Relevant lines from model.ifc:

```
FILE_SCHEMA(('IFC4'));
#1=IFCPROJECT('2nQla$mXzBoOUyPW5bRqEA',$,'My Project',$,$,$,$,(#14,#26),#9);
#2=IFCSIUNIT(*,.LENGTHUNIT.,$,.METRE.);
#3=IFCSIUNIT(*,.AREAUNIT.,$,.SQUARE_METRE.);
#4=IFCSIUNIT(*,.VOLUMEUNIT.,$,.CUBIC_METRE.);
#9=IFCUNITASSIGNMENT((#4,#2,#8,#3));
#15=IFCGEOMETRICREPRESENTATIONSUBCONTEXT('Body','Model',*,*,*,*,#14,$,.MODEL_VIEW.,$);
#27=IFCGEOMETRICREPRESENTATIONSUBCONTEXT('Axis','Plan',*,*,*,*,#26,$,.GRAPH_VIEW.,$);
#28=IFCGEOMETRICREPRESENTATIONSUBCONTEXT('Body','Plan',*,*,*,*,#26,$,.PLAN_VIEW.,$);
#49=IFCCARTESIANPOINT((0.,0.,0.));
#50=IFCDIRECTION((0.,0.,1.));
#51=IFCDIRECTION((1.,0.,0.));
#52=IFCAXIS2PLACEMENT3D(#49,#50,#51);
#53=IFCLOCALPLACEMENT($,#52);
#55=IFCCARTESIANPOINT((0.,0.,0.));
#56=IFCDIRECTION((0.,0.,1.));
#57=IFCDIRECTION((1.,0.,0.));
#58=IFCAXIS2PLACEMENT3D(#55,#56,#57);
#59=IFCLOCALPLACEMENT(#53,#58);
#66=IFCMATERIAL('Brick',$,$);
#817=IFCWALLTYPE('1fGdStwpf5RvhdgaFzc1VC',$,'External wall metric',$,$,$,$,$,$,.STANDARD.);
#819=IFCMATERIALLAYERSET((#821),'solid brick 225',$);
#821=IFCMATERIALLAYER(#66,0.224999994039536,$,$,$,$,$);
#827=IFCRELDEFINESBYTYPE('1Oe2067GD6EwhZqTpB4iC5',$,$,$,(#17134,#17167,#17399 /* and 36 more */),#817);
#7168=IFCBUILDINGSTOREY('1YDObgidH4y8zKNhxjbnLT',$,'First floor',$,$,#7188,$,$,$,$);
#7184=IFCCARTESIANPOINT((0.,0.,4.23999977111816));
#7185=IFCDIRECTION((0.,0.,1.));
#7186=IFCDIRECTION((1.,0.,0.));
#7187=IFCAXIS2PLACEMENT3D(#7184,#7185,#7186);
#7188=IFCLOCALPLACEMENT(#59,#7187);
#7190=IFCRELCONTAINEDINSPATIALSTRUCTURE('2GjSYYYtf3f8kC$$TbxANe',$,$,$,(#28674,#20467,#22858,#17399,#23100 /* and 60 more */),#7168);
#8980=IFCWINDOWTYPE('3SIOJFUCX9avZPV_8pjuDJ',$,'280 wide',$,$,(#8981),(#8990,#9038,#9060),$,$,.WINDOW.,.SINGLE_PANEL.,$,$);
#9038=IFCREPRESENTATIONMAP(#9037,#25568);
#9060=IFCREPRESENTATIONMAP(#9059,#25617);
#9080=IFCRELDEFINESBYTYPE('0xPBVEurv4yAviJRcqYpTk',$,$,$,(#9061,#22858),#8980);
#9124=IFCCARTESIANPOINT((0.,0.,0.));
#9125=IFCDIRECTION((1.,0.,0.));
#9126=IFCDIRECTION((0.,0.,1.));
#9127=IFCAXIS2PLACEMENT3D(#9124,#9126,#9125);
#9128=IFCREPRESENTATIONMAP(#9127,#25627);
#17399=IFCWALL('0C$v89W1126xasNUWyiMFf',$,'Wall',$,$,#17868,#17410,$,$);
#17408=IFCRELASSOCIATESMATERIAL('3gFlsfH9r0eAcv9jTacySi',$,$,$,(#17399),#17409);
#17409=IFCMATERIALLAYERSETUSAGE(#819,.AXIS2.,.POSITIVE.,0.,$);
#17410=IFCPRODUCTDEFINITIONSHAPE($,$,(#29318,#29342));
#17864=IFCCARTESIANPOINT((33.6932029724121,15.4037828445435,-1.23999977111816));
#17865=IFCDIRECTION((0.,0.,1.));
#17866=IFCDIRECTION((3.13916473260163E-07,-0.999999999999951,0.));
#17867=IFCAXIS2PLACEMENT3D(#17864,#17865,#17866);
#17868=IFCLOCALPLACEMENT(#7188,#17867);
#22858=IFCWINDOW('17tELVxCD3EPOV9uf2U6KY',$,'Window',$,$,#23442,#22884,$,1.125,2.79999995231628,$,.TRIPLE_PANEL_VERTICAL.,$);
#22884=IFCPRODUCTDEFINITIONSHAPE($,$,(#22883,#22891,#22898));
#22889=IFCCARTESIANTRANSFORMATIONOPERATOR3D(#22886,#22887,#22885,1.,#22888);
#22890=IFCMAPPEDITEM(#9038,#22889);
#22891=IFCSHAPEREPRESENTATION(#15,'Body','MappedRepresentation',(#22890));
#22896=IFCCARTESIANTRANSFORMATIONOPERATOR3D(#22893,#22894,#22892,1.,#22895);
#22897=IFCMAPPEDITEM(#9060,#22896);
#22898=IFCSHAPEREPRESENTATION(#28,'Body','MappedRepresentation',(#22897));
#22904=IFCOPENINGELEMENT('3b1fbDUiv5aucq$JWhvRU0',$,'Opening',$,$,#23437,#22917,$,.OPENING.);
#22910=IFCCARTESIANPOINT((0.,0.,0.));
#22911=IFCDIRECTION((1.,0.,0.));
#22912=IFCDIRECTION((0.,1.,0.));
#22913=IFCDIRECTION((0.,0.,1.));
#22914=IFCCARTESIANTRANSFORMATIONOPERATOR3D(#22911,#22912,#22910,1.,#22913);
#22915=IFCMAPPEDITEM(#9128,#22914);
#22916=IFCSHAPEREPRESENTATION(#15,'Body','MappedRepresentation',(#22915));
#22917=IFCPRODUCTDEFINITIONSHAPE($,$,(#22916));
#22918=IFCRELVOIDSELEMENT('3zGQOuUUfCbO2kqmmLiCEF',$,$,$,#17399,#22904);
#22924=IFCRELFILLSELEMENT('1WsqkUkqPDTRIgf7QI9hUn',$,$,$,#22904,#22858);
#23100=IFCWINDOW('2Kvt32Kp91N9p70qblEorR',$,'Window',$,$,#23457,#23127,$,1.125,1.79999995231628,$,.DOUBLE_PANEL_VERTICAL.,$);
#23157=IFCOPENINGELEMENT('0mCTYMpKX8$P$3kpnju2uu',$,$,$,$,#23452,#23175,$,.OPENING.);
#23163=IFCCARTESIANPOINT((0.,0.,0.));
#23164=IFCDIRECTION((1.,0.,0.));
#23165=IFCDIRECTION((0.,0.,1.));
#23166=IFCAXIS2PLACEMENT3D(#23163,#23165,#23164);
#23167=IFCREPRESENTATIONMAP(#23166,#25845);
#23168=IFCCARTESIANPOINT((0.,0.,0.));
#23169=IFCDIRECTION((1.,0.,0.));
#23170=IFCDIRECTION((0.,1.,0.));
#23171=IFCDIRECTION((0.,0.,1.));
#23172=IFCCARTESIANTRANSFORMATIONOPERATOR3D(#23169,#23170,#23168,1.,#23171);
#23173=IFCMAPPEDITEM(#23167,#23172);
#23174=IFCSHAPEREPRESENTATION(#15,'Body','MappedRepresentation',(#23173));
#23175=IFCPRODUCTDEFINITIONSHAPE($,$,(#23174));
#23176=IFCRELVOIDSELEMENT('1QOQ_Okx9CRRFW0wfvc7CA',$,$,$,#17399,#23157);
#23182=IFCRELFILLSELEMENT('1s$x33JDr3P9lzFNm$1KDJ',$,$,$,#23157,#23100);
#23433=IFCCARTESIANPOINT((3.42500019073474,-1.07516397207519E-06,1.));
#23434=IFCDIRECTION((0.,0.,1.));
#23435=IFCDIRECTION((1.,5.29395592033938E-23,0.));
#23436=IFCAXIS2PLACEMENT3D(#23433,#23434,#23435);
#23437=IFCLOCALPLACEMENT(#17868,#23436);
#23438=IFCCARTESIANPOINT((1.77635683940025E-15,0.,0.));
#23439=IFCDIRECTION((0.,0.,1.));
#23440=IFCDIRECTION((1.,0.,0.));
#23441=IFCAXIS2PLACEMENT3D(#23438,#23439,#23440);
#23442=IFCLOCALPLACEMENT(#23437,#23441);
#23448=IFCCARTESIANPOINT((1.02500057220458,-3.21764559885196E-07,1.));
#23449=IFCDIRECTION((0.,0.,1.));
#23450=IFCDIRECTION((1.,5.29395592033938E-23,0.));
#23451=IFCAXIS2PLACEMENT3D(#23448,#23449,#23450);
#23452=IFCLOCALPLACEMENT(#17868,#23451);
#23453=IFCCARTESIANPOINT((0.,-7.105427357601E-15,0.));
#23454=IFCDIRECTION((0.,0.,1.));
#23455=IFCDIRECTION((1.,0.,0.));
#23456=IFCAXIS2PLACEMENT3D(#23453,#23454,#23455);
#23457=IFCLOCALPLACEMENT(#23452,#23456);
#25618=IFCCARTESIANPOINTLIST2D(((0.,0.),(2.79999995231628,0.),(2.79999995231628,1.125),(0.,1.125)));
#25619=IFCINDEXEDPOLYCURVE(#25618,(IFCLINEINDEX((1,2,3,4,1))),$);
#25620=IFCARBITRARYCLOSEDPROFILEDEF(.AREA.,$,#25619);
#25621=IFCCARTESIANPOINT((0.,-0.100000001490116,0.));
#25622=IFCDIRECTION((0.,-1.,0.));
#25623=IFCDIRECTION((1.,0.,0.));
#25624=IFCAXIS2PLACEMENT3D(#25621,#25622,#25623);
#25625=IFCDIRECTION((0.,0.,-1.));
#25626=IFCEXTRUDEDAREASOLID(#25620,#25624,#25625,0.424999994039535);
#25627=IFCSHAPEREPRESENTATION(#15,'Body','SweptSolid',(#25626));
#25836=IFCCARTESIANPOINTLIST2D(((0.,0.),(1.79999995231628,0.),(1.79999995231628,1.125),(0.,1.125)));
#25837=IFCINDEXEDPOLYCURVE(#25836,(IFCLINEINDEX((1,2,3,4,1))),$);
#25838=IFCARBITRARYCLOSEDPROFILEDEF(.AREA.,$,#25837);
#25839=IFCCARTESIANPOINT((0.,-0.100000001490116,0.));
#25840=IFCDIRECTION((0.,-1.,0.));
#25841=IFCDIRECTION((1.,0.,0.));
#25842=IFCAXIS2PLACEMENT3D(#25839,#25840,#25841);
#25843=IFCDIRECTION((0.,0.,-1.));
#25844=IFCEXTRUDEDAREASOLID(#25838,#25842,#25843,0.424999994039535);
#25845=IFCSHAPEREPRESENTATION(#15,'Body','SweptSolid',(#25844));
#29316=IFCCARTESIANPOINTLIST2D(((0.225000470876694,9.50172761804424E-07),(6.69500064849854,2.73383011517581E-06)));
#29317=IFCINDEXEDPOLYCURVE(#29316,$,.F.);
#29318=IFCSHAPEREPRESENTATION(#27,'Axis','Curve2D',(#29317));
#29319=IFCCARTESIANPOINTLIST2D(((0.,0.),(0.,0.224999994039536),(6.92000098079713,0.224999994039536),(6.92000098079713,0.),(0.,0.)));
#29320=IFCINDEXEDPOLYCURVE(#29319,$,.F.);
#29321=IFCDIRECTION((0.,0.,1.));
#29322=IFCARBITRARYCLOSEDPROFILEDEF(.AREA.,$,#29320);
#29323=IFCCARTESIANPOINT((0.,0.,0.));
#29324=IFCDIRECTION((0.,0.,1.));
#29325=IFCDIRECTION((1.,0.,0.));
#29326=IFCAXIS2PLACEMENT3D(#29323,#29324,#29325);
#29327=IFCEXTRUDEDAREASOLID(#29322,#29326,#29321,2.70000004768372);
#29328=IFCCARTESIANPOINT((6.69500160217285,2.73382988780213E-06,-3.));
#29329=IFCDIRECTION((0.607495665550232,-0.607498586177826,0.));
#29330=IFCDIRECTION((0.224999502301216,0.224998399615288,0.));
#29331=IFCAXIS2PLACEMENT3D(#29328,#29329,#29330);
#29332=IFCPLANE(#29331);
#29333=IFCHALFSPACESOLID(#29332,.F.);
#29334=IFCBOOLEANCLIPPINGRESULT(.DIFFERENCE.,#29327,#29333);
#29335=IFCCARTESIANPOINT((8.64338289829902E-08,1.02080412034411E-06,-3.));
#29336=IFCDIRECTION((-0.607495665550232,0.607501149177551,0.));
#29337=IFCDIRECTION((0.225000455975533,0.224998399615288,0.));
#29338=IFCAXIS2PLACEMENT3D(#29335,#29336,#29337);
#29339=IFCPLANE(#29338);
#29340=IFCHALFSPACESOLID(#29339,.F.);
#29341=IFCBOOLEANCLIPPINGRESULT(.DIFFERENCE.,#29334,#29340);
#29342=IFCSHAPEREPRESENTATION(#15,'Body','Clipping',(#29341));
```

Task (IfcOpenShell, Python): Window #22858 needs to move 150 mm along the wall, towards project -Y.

```python
import ifcopenshell
import ifcopenshell.api.geometry
import ifcopenshell.util.placement
import ifcopenshell.util.unit

model = ifcopenshell.open("model.ifc")
unit_scale = ifcopenshell.util.unit.calculate_unit_scale(model)

window = model.by_guid("17tELVxCD3EPOV9uf2U6KY")
opening = window.FillsVoids[0].RelatingOpeningElement
wall = opening.VoidsElements[0].RelatingBuildingElement

wall_matrix = ifcopenshell.util.placement.get_local_placement(wall.ObjectPlacement)
shift = wall_matrix[:3, 0] * 0.15 / unit_scale
before = ifcopenshell.util.placement.get_local_placement(window.ObjectPlacement)[:3, 3].copy()

# The window is placed relative to its opening, so it follows when the opening moves.
matrix = ifcopenshell.util.placement.get_local_placement(opening.ObjectPlacement)
matrix[:3, 3] += shift
ifcopenshell.api.geometry.edit_object_placement(
    model, product=opening, matrix=matrix, is_si=False, should_transform_children=True
)

after = ifcopenshell.util.placement.get_local_placement(window.ObjectPlacement)[:3, 3]
print("window moved by", (after - before).round(3) + 0.0)

model.write("model_v2.ifc")
```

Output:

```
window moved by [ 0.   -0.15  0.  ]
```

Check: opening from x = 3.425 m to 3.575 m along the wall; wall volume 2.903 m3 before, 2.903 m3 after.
